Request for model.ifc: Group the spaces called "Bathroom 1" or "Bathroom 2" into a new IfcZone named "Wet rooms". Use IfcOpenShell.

First a look at what the model holds.

```python
import ifcopenshell

model = ifcopenshell.open("model.ifc")
print(model.schema)
seen = {}
for space in model.by_type("IfcSpace"):
    seen[space.LongName] = seen.get(space.LongName, 0) + 1
for name, count in sorted(seen.items(), key=str):
    print(count, "x", name)
print("zones:", [z.Name for z in model.by_type("IfcZone")][:20])
```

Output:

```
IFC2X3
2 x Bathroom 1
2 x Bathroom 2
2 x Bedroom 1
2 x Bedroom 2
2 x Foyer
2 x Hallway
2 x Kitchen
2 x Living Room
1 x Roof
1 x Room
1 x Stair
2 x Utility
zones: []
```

```python
import ifcopenshell
import ifcopenshell.api.group
import ifcopenshell.api.root

model = ifcopenshell.open("model.ifc")

names = {"Bathroom 1", "Bathroom 2"}
spaces = [s for s in model.by_type("IfcSpace") if s.LongName in names]

zone = ifcopenshell.api.root.create_entity(model, ifc_class="IfcZone", name="Wet rooms")
ifcopenshell.api.group.assign_group(model, products=spaces, group=zone)
print(len(spaces), "spaces in", zone.Name)

model.write("model_edited.ifc")
```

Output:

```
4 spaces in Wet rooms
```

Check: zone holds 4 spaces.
